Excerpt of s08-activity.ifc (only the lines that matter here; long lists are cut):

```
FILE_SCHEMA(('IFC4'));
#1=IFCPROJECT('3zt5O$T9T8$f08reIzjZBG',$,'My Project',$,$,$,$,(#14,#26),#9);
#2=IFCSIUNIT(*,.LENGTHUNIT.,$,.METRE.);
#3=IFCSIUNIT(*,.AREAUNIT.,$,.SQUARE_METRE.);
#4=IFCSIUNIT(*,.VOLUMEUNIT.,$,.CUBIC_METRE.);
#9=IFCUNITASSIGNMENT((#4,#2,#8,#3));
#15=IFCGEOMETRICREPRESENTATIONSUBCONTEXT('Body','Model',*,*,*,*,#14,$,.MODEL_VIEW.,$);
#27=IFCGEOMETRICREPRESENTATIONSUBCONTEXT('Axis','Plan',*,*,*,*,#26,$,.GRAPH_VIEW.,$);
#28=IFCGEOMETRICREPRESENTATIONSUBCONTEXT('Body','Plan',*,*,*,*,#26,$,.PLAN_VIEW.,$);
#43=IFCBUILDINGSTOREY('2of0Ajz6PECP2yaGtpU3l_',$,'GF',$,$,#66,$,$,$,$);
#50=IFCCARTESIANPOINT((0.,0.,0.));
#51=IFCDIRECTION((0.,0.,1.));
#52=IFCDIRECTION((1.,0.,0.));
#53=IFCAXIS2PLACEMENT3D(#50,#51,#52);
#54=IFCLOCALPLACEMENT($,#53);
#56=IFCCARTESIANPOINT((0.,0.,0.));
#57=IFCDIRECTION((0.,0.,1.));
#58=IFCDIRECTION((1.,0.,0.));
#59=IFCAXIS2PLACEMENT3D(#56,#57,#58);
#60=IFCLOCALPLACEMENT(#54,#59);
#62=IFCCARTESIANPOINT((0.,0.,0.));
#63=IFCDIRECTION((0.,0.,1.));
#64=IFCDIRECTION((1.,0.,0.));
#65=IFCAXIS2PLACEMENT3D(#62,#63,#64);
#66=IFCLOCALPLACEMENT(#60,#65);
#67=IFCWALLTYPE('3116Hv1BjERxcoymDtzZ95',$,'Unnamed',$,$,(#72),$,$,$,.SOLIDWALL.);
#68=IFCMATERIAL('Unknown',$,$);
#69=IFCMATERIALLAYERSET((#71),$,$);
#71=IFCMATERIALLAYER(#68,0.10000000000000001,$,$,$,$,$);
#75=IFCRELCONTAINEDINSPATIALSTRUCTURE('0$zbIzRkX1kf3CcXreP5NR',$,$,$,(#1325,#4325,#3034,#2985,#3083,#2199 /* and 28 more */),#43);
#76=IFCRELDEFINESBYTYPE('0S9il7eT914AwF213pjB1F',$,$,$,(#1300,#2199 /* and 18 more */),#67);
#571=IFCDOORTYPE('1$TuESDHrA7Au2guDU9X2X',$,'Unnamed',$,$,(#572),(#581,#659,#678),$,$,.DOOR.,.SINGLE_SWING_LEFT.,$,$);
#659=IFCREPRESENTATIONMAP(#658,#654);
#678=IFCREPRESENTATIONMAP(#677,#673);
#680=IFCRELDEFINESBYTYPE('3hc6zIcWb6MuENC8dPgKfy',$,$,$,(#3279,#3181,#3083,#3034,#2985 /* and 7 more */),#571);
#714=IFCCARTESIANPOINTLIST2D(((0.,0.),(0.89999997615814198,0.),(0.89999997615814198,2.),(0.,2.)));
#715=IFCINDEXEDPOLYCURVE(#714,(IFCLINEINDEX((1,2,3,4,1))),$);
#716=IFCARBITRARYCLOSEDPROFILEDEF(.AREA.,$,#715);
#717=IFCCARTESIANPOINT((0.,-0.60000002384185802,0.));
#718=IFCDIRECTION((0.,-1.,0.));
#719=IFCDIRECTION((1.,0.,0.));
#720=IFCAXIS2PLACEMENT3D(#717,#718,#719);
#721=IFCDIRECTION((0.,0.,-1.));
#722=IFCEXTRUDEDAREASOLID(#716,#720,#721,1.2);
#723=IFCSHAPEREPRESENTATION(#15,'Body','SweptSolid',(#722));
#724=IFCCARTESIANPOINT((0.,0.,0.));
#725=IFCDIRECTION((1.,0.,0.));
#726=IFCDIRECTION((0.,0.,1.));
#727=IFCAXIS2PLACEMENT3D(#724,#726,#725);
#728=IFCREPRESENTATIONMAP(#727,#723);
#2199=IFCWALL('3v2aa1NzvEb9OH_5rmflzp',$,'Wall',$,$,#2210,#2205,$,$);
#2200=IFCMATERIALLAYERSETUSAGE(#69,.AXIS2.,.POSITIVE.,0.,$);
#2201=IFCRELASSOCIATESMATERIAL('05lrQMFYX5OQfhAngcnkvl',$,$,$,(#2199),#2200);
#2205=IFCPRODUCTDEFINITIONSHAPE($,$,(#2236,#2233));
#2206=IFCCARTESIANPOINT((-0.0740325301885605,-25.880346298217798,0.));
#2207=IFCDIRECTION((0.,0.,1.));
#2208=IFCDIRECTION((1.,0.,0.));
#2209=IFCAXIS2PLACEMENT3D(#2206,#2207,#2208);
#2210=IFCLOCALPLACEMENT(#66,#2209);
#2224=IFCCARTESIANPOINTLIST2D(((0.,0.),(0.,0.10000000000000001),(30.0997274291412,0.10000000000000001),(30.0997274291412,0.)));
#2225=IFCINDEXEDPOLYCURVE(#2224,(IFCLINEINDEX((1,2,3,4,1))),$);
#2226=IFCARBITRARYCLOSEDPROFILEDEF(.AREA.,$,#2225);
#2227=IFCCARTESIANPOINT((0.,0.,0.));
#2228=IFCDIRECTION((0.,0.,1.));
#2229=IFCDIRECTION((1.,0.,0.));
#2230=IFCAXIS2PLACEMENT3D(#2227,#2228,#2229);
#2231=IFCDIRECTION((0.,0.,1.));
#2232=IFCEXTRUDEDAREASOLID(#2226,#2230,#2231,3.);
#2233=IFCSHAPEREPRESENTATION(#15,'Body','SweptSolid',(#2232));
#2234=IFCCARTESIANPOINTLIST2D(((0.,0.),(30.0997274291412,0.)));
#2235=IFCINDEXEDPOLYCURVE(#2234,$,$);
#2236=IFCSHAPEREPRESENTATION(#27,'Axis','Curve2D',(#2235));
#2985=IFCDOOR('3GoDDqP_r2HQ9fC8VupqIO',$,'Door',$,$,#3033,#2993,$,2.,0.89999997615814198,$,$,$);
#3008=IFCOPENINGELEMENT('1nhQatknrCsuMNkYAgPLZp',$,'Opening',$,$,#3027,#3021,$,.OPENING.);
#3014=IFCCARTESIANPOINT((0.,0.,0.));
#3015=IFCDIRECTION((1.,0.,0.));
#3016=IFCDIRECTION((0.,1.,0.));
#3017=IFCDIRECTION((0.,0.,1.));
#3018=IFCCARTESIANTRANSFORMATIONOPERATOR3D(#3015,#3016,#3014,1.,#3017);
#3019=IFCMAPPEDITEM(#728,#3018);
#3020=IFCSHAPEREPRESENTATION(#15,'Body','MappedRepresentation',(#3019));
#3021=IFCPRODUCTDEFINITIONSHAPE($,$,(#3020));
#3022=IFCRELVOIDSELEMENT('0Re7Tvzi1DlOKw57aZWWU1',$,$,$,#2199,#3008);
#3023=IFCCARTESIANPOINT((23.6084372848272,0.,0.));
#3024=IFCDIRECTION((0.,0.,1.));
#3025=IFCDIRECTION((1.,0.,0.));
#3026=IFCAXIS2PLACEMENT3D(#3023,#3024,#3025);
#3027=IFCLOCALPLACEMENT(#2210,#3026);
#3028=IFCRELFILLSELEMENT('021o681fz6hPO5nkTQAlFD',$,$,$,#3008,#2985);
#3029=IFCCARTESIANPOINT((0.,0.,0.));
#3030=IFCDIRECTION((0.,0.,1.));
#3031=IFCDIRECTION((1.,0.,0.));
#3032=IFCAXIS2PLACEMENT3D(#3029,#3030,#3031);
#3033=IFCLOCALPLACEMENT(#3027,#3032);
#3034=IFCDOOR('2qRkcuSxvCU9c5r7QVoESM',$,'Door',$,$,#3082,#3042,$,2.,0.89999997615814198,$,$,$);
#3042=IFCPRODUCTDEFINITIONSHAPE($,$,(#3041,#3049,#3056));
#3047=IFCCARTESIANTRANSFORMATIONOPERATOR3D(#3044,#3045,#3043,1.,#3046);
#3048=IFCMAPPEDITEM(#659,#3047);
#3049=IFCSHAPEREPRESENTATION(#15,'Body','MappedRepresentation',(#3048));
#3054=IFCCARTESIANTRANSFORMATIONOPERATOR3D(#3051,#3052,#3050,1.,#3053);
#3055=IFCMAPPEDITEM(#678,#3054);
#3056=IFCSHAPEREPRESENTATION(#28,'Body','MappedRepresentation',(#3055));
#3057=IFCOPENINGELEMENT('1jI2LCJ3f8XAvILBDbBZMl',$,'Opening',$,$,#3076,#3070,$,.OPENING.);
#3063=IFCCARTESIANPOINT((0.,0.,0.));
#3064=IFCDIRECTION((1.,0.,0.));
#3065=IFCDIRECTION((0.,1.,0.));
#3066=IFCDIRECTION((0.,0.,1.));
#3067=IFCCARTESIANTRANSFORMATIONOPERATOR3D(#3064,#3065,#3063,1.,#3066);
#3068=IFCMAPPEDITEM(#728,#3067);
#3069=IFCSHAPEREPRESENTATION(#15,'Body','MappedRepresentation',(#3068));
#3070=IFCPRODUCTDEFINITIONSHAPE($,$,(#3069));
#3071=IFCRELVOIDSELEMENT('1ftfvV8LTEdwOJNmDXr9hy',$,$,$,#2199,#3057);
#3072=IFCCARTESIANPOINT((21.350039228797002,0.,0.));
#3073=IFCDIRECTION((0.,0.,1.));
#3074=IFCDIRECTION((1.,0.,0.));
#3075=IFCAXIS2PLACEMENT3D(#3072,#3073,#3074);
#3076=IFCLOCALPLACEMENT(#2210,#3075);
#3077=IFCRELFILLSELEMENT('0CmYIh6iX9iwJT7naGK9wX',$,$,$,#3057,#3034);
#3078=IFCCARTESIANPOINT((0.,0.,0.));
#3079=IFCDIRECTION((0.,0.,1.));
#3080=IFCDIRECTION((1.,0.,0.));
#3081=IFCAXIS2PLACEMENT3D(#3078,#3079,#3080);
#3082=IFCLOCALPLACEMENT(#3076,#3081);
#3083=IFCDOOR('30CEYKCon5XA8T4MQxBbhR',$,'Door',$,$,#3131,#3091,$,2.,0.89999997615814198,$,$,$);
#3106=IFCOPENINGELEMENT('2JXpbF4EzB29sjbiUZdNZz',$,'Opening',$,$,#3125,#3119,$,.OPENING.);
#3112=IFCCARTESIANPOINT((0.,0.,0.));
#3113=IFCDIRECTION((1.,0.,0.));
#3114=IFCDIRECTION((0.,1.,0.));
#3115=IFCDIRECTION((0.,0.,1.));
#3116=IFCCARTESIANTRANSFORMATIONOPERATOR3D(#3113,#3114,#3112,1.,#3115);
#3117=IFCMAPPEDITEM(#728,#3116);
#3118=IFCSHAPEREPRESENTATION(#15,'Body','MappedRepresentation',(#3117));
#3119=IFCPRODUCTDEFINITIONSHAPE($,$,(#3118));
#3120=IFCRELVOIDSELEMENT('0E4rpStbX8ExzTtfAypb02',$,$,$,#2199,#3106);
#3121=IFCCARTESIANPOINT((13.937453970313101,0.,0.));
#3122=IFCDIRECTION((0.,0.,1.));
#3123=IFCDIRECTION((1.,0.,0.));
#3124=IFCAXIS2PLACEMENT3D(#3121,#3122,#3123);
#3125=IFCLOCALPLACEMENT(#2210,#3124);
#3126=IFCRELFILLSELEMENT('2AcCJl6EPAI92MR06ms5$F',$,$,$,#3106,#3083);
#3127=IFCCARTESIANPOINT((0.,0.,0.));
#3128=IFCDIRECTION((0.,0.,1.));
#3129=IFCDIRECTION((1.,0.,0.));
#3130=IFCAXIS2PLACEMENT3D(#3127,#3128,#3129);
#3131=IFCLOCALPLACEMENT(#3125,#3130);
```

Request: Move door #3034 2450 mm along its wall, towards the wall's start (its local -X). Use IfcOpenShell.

```python
import ifcopenshell
import ifcopenshell.api.geometry
import ifcopenshell.util.placement

model = ifcopenshell.open("s08-activity.ifc")

door = model.by_guid("2qRkcuSxvCU9c5r7QVoESM")
opening = door.FillsVoids[0].RelatingOpeningElement
wall = opening.VoidsElements[0].RelatingBuildingElement

wall_matrix = ifcopenshell.util.placement.get_local_placement(wall.ObjectPlacement)
shift = wall_matrix[:3, 0] * -2.45
before = ifcopenshell.util.placement.get_local_placement(door.ObjectPlacement)[:3, 3].copy()

# The door is placed relative to its opening, so it follows when the opening moves.
matrix = ifcopenshell.util.placement.get_local_placement(opening.ObjectPlacement)
matrix[:3, 3] += shift
ifcopenshell.api.geometry.edit_object_placement(
    model, product=opening, matrix=matrix, is_si=False, should_transform_children=True
)

after = ifcopenshell.util.placement.get_local_placement(door.ObjectPlacement)[:3, 3]
print("door moved by", (after - before).round(3) + 0.0)

model.write("s08-activity-out.ifc")
```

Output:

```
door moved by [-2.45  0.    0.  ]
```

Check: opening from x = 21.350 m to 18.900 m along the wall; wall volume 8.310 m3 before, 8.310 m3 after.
